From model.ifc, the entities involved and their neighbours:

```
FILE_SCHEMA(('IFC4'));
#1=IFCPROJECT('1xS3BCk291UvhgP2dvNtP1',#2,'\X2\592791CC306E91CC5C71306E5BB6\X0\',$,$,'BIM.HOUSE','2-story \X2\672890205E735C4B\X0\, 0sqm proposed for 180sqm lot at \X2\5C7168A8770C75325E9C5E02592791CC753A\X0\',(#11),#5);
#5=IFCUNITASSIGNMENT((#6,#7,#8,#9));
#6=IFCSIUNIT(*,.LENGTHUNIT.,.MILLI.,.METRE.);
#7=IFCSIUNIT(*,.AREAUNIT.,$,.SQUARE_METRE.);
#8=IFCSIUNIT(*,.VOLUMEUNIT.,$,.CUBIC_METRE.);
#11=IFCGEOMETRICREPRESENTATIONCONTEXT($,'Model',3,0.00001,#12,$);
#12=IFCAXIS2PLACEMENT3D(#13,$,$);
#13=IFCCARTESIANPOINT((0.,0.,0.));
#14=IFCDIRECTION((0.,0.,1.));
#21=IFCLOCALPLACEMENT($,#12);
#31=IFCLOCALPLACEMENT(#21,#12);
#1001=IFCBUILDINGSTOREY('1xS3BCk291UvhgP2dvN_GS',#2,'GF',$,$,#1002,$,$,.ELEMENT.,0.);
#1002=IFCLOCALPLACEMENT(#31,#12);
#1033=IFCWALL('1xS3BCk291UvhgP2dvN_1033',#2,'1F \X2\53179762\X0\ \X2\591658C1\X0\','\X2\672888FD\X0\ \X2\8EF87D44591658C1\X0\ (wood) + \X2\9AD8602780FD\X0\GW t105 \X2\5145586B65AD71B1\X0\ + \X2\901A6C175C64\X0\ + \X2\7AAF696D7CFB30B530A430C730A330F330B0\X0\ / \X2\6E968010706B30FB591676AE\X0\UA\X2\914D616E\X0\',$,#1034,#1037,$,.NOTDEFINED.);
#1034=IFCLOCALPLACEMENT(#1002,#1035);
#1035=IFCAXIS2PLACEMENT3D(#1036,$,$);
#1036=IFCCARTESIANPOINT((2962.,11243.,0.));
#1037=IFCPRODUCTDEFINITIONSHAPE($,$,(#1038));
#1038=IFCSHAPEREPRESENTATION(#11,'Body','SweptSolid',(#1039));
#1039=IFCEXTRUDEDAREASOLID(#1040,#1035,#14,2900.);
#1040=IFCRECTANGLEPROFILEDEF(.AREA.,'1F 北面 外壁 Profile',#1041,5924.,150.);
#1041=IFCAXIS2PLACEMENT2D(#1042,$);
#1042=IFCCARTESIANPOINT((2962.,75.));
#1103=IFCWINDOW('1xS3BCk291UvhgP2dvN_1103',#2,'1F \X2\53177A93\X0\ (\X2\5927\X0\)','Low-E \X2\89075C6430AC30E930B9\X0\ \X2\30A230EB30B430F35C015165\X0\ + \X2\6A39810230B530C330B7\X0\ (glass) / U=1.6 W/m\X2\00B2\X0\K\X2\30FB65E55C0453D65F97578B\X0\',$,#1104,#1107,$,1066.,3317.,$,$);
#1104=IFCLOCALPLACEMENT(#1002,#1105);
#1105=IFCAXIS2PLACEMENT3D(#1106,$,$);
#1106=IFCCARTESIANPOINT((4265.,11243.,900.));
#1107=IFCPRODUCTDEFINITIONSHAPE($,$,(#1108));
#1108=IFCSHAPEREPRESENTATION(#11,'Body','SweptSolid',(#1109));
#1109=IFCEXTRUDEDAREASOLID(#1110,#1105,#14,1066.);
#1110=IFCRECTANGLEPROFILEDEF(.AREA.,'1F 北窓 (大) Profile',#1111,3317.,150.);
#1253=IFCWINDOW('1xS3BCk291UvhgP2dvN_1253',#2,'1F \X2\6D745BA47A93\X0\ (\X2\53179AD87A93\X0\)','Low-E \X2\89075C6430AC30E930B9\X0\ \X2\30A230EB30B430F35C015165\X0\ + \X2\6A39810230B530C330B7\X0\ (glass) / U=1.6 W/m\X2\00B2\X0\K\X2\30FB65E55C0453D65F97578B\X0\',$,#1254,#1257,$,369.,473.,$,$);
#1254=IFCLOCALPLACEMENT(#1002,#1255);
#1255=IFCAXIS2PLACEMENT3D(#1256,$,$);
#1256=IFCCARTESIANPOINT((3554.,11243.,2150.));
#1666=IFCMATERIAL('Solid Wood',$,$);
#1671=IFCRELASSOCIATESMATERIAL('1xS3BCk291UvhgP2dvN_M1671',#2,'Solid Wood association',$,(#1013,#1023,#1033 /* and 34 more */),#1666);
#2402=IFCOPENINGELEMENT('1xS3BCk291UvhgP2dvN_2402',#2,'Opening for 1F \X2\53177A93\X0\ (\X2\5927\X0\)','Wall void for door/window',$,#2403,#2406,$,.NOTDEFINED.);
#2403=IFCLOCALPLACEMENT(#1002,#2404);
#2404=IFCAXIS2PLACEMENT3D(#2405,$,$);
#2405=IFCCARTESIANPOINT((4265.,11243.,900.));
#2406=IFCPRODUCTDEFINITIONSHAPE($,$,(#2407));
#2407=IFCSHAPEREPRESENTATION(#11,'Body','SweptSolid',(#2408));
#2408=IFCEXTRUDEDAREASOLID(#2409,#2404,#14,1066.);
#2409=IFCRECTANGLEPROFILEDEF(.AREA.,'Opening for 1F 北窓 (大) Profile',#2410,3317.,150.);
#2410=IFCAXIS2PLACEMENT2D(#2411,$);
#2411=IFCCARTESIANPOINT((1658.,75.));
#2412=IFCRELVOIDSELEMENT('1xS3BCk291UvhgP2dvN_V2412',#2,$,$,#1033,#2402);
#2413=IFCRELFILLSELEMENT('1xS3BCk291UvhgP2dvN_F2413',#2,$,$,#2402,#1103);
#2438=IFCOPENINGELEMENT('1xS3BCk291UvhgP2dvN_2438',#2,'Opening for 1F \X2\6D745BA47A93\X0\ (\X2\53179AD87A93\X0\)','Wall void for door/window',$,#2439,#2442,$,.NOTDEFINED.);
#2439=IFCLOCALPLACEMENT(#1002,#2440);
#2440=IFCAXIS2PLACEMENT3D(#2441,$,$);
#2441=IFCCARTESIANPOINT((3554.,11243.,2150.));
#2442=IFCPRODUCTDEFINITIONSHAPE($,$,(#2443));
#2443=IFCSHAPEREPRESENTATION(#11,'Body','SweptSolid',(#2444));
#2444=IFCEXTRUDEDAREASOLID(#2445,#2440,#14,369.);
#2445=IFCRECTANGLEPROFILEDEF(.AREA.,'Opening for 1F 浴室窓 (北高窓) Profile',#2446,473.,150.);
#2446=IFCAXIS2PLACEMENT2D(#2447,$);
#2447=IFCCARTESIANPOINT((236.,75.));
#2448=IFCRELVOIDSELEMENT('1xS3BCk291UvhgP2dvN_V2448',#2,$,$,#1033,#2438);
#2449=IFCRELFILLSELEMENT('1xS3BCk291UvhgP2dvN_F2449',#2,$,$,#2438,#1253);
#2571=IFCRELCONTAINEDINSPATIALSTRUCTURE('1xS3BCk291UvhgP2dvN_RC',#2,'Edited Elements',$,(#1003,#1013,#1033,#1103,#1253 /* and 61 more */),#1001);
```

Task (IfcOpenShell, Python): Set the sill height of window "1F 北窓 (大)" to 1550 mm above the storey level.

```python
import numpy as np
import ifcopenshell
import ifcopenshell.api.geometry
import ifcopenshell.geom
import ifcopenshell.util.element
import ifcopenshell.util.placement
import ifcopenshell.util.shape
import ifcopenshell.util.unit

model = ifcopenshell.open("model.ifc")
unit_scale = ifcopenshell.util.unit.calculate_unit_scale(model)

window = model.by_id(1103)
opening = window.FillsVoids[0].RelatingOpeningElement
storey = ifcopenshell.util.element.get_container(window, ifc_class="IfcBuildingStorey")
level = ifcopenshell.util.placement.get_local_placement(storey.ObjectPlacement)[2, 3]

# The opening's origin need not be at the sill, so measure its lowest point.
shape = ifcopenshell.geom.create_shape(ifcopenshell.geom.settings(), opening)
bottom = ifcopenshell.util.shape.get_shape_bottom_elevation(shape, shape.geometry) / unit_scale
dz = level + 1.55 / unit_scale - bottom

shift = np.array([0.0, 0.0, dz])
# The window is not placed relative to its opening, so move both.
for product in (opening, window):
    matrix = ifcopenshell.util.placement.get_local_placement(product.ObjectPlacement)
    matrix[:3, 3] += shift
    ifcopenshell.api.geometry.edit_object_placement(model, product=product, matrix=matrix, is_si=False)

print(f"moved by {dz * unit_scale:+.3f} m")

model.write("model-out.ifc")
```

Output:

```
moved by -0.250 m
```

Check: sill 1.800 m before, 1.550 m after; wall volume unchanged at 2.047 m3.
